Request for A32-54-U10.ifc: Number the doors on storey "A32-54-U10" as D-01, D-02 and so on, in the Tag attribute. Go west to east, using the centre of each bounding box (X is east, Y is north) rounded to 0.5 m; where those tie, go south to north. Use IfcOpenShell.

First a look at what the model holds.

```python
import ifcopenshell
import ifcopenshell.util.element
import ifcopenshell.util.placement

model = ifcopenshell.open("A32-54-U10.ifc")
print(model.schema)
storey = next(s for s in model.by_type("IfcBuildingStorey") if s.Name == "A32-54-U10")
doors = [e for e in ifcopenshell.util.element.get_decomposition(storey) if e.is_a("IfcDoor")]
for e in sorted(doors, key=lambda e: e.id()):
    origin = ifcopenshell.util.placement.get_local_placement(e.ObjectPlacement)[:3, 3]
    print(e.id(), e.Tag, e.Name, origin.round(2) + 0.0, sep=" | ")
```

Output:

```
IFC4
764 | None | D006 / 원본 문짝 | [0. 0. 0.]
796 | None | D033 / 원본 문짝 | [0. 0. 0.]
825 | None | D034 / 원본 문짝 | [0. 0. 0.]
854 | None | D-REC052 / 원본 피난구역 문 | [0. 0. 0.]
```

```python
import ifcopenshell
import ifcopenshell.geom
import ifcopenshell.util.element
import ifcopenshell.util.shape

model = ifcopenshell.open("A32-54-U10.ifc")
settings = ifcopenshell.geom.settings()
settings.set("use-world-coords", True)


def centre(element):
    shape = ifcopenshell.geom.create_shape(settings, element)
    return ifcopenshell.util.shape.get_bbox_centroid(shape.geometry)


storey = next(s for s in model.by_type("IfcBuildingStorey") if s.Name == "A32-54-U10")
doors = [e for e in ifcopenshell.util.element.get_decomposition(storey) if e.is_a("IfcDoor")]

# Insertion points can sit at a corner or the storey origin, so sort by the geometry (in metres).
centres = {e: centre(e) for e in doors}
doors.sort(key=lambda e: (round(centres[e][0] / 0.5), centres[e][1]))

for i, e in enumerate(doors, start=1):
    number = f"D-{i:02d}"
    e.Tag = number
    print(e.id(), number)

model.write("A32-54-U10_v2.ifc")
```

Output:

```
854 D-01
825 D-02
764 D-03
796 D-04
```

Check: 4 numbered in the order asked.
